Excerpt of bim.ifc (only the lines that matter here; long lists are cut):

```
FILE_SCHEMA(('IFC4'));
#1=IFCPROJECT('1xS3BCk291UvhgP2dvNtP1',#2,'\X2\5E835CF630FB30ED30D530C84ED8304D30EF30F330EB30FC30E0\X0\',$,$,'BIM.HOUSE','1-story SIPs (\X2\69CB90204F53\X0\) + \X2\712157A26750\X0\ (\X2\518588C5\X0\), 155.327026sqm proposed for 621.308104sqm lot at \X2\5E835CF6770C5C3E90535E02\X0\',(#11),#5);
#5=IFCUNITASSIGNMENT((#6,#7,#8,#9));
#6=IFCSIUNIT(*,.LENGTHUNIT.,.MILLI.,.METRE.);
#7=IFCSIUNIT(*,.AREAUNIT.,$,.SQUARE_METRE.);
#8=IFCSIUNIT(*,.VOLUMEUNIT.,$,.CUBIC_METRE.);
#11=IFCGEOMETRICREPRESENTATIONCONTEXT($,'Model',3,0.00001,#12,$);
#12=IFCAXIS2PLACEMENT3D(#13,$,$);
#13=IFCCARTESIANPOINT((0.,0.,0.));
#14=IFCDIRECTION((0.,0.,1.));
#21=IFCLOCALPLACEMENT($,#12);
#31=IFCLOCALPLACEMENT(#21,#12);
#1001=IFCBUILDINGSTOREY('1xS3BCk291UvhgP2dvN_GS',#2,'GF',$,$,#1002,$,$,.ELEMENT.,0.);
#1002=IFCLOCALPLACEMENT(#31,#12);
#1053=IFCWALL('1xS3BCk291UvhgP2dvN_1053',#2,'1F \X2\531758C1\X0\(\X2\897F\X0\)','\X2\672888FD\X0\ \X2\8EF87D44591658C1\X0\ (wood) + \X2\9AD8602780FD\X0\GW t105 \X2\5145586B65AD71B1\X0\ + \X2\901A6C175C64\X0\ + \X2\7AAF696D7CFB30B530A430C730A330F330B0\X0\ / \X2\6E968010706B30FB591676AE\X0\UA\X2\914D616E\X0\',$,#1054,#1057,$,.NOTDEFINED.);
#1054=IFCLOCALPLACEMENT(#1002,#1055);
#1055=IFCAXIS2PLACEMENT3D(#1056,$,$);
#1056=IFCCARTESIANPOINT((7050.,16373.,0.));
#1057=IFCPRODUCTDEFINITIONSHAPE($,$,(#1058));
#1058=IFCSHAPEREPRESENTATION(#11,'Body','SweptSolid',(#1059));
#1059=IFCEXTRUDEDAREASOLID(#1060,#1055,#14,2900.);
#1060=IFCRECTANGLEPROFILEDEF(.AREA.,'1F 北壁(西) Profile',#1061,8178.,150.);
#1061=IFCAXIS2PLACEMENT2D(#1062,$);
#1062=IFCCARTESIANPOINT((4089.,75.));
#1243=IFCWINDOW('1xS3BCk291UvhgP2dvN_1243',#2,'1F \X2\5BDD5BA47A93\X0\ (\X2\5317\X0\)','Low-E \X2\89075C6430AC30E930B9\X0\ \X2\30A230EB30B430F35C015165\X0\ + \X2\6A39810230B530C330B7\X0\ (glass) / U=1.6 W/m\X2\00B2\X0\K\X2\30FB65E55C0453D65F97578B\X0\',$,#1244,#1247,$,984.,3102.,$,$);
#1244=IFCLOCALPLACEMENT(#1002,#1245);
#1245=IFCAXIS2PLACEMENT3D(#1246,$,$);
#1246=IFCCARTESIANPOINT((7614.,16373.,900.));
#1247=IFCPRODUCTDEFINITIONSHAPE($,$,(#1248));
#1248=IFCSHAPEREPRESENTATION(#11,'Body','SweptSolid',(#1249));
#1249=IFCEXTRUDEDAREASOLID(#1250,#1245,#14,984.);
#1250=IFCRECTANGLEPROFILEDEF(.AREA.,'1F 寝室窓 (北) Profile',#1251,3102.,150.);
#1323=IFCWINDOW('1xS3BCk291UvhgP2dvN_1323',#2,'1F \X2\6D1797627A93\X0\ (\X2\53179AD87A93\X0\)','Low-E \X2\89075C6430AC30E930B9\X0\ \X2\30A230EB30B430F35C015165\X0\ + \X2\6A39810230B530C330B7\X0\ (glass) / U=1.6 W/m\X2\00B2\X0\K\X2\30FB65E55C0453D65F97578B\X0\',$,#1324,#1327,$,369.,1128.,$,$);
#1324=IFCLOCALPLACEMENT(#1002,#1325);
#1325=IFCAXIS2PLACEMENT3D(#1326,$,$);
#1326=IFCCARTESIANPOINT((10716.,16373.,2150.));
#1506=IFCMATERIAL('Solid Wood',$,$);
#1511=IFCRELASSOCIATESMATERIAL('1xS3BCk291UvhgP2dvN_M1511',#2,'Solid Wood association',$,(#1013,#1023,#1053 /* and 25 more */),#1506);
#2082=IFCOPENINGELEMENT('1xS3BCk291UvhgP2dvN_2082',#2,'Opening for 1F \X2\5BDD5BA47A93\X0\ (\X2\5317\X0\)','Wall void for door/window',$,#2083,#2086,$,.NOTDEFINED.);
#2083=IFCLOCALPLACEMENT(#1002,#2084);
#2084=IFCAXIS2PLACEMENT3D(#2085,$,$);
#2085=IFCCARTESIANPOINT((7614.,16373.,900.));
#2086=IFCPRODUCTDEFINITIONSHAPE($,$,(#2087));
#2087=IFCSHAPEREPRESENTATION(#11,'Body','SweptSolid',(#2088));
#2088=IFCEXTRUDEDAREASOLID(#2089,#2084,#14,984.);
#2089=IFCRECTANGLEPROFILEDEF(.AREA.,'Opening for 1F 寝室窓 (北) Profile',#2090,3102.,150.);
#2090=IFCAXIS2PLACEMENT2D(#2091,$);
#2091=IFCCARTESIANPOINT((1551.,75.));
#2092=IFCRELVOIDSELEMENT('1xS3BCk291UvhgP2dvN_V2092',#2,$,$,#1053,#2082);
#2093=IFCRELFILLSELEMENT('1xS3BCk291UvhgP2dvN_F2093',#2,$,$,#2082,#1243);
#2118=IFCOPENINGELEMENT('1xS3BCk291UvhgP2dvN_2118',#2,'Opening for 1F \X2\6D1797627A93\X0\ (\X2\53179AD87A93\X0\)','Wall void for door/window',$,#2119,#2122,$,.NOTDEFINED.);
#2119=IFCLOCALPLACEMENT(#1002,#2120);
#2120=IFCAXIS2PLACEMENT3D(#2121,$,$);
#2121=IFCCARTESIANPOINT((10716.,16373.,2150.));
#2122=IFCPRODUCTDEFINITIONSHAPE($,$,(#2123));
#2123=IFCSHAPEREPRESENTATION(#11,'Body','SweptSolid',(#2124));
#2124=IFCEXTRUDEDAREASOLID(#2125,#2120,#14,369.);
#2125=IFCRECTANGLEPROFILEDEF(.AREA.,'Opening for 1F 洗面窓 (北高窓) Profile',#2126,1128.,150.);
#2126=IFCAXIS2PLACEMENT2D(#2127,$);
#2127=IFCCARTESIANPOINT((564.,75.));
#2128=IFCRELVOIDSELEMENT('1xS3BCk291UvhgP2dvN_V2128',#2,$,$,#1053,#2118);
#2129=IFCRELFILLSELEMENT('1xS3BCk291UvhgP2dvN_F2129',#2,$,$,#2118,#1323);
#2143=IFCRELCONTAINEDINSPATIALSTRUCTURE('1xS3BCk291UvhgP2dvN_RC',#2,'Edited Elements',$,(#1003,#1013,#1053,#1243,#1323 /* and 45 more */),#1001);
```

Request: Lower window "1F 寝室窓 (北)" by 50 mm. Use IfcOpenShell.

```python
import numpy as np
import ifcopenshell
import ifcopenshell.api.geometry
import ifcopenshell.util.placement
import ifcopenshell.util.unit

model = ifcopenshell.open("bim.ifc")
unit_scale = ifcopenshell.util.unit.calculate_unit_scale(model)

window = model.by_id(1243)
opening = window.FillsVoids[0].RelatingOpeningElement
dz = -50.0

shift = np.array([0.0, 0.0, dz])
# The window is not placed relative to its opening, so move both.
for product in (opening, window):
    matrix = ifcopenshell.util.placement.get_local_placement(product.ObjectPlacement)
    matrix[:3, 3] += shift
    ifcopenshell.api.geometry.edit_object_placement(model, product=product, matrix=matrix, is_si=False)

print(f"moved by {dz * unit_scale:+.3f} m")

model.write("bim_rev.ifc")
```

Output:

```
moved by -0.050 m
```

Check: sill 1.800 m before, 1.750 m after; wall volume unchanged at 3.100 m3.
